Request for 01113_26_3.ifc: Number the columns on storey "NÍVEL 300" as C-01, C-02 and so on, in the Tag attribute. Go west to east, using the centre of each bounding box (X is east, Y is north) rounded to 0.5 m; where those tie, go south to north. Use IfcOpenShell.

First a look at what the model holds.

```python
import ifcopenshell
import ifcopenshell.util.element
import ifcopenshell.util.placement

model = ifcopenshell.open("01113_26_3.ifc")
print(model.schema)
storey = next(s for s in model.by_type("IfcBuildingStorey") if s.Name == "NÍVEL 300")
columns = [e for e in ifcopenshell.util.element.get_decomposition(storey) if e.is_a("IfcColumn")]
for e in sorted(columns, key=lambda e: e.id()):
    origin = ifcopenshell.util.placement.get_local_placement(e.ObjectPlacement)[:3, 3]
    print(e.id(), e.Tag, e.Name, origin.round(2) + 0.0, sep=" | ")
```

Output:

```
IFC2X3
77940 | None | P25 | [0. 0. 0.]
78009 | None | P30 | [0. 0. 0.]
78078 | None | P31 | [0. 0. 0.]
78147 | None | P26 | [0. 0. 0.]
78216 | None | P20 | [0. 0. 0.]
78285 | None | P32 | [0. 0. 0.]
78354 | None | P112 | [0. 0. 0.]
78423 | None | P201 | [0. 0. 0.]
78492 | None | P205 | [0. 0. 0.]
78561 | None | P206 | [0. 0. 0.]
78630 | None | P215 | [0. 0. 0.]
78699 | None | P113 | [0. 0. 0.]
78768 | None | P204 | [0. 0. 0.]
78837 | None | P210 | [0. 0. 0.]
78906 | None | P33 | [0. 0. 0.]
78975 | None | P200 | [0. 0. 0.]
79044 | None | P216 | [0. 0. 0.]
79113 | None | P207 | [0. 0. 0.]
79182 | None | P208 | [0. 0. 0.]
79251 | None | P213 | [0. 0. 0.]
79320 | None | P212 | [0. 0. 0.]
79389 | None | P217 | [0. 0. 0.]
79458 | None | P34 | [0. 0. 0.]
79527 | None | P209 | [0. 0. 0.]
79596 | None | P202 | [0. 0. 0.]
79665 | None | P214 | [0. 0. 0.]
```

```python
import ifcopenshell
import ifcopenshell.geom
import ifcopenshell.util.element
import ifcopenshell.util.shape

model = ifcopenshell.open("01113_26_3.ifc")
settings = ifcopenshell.geom.settings()
settings.set("use-world-coords", True)


def centre(element):
    shape = ifcopenshell.geom.create_shape(settings, element)
    return ifcopenshell.util.shape.get_bbox_centroid(shape.geometry)


storey = next(s for s in model.by_type("IfcBuildingStorey") if s.Name == "NÍVEL 300")
columns = [e for e in ifcopenshell.util.element.get_decomposition(storey) if e.is_a("IfcColumn")]

# Insertion points can sit at a corner or the storey origin, so sort by the geometry (in metres).
centres = {e: centre(e) for e in columns}
columns.sort(key=lambda e: (round(centres[e][0] / 0.5), centres[e][1]))

for i, e in enumerate(columns, start=1):
    number = f"C-{i:02d}"
    e.Tag = number
    print(e.id(), number)

model.write("01113_26_3_edited.ifc")
```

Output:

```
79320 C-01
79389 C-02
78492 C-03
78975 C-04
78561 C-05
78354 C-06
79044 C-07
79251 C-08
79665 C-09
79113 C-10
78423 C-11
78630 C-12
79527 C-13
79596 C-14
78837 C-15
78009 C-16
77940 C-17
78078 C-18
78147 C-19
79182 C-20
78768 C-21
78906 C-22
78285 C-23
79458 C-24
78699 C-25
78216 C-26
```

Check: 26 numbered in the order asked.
